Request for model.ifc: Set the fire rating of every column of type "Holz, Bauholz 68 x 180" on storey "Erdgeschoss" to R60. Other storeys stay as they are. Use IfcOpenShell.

First a look at what the model holds.

```python
import ifcopenshell
import ifcopenshell.util.element

model = ifcopenshell.open("model.ifc")
print(model.schema)
storey = next(s for s in model.by_type("IfcBuildingStorey") if s.Name == "Erdgeschoss")
columns = [e for e in ifcopenshell.util.element.get_decomposition(storey) if e.is_a("IfcColumn")]
seen = {}
for e in columns:
    element_type = ifcopenshell.util.element.get_type(e)
    key = (element_type.Name if element_type != e and element_type else None, ifcopenshell.util.element.get_pset(e, "Pset_ColumnCommon", "FireRating"))
    seen[key] = seen.get(key, 0) + 1
for (name, value), count in sorted(seen.items(), key=str):
    print(count, "x", name, "|", value)
```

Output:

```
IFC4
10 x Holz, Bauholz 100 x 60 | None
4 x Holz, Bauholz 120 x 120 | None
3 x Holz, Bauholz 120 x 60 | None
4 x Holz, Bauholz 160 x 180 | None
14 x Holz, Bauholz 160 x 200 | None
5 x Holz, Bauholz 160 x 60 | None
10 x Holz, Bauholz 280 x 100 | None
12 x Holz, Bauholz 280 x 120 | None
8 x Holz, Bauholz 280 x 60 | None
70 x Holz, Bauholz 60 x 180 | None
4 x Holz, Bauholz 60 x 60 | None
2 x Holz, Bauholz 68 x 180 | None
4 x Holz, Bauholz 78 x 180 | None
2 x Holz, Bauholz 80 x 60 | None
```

```python
import ifcopenshell
import ifcopenshell.api.pset
import ifcopenshell.util.element

model = ifcopenshell.open("model.ifc")

storey = next(s for s in model.by_type("IfcBuildingStorey") if s.Name == "Erdgeschoss")
columns = [e for e in ifcopenshell.util.element.get_decomposition(storey) if e.is_a("IfcColumn")]

count = 0
for e in columns:
    element_type = ifcopenshell.util.element.get_type(e)
    if element_type in (None, e) or element_type.Name != "Holz, Bauholz 68 x 180":
        continue
    # add_pset returns the element's existing set when there is one.
    pset = ifcopenshell.api.pset.add_pset(model, product=e, name="Pset_ColumnCommon")
    ifcopenshell.api.pset.edit_pset(model, pset=pset, properties={"FireRating": "R60"})
    count += 1

print(count, "columns updated")

model.write("model-out.ifc")
```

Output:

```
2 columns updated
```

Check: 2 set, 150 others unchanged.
